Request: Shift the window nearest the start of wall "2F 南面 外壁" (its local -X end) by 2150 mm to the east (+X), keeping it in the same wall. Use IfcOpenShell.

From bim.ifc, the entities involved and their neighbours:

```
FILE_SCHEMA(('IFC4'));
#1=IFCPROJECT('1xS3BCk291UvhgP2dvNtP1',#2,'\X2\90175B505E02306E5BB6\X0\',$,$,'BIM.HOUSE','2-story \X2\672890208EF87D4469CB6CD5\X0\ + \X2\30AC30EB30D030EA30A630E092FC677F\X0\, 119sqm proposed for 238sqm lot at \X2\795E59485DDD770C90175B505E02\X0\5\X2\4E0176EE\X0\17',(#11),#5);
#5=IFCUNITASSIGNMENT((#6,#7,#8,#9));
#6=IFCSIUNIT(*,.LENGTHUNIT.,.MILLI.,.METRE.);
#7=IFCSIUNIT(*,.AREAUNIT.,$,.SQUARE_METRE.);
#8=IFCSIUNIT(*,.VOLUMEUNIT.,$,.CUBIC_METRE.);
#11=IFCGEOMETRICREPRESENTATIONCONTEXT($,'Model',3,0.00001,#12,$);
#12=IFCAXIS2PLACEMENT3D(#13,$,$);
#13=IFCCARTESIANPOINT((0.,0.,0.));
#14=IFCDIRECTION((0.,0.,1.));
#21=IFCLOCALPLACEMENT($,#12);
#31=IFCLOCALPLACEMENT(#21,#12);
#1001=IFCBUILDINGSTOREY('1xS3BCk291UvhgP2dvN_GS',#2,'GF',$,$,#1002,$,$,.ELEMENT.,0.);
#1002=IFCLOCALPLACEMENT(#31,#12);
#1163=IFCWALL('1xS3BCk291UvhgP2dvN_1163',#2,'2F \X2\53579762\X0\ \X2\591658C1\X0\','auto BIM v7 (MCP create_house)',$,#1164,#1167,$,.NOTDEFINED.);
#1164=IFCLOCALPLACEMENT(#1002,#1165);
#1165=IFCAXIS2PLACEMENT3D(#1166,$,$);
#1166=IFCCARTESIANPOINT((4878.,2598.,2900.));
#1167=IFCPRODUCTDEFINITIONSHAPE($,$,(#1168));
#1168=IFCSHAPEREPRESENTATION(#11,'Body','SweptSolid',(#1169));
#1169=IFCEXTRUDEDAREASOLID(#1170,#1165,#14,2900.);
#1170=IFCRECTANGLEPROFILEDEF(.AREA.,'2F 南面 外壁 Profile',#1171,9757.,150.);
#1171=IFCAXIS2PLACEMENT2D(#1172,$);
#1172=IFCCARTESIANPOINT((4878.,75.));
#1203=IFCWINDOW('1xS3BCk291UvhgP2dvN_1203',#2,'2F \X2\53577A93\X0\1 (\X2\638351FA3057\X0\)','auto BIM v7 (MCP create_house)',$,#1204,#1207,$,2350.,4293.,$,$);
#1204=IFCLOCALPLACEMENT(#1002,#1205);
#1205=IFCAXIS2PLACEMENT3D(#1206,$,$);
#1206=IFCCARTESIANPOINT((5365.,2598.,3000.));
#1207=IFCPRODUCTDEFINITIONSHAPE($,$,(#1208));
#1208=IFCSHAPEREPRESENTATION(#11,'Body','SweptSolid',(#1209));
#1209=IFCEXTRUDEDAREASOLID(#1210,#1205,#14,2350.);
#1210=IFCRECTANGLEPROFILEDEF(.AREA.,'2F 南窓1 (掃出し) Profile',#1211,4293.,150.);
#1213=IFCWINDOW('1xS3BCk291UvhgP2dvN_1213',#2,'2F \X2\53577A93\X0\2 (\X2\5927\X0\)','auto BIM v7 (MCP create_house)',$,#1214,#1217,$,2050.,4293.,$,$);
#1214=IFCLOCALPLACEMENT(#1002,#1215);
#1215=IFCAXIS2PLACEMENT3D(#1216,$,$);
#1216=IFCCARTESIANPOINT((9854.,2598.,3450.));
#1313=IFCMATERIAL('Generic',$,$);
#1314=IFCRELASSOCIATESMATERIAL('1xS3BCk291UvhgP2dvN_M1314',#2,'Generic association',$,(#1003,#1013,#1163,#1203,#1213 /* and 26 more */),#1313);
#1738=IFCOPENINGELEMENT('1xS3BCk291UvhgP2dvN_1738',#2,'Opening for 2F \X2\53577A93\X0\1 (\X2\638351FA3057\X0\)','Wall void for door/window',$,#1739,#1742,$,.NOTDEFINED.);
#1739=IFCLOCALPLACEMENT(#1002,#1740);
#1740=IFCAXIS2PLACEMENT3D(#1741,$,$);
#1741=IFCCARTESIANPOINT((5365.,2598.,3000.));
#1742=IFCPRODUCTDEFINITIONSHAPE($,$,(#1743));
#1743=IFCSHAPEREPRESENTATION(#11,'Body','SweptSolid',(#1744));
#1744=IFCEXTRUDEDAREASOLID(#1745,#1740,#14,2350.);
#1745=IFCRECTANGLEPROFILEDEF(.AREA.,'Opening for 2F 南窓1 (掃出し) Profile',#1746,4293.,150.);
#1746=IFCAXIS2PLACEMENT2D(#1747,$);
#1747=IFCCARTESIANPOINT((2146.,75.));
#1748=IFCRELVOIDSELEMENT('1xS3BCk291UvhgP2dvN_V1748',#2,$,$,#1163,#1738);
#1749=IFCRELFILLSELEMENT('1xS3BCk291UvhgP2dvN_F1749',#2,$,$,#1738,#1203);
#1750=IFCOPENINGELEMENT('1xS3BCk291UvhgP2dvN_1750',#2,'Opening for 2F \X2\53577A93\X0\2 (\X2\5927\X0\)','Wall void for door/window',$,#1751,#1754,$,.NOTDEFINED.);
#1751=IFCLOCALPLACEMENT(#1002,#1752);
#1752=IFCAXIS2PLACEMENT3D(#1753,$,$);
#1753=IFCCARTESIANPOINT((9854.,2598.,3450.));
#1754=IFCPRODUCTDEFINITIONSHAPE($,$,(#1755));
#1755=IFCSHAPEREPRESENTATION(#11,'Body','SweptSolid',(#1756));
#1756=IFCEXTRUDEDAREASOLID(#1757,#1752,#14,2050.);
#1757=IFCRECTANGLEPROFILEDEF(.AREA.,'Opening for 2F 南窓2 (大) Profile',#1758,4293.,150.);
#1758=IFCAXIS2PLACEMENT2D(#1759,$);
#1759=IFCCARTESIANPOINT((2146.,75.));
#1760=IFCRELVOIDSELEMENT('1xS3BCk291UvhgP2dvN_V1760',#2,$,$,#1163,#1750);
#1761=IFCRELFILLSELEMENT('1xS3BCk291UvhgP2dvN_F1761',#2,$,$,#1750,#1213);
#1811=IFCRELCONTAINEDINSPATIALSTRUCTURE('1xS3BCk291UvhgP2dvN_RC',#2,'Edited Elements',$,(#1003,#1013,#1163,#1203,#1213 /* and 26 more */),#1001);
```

```python
import ifcopenshell
import ifcopenshell.api.geometry
import ifcopenshell.util.placement
import ifcopenshell.util.unit

model = ifcopenshell.open("bim.ifc")
unit_scale = ifcopenshell.util.unit.calculate_unit_scale(model)

window = model.by_guid("1xS3BCk291UvhgP2dvN_1203")
opening = window.FillsVoids[0].RelatingOpeningElement
wall = opening.VoidsElements[0].RelatingBuildingElement

wall_matrix = ifcopenshell.util.placement.get_local_placement(wall.ObjectPlacement)
shift = wall_matrix[:3, 0] * 2.15 / unit_scale
before = ifcopenshell.util.placement.get_local_placement(window.ObjectPlacement)[:3, 3].copy()

# The window is not placed relative to its opening, so move both.
for product in (opening, window):
    matrix = ifcopenshell.util.placement.get_local_placement(product.ObjectPlacement)
    matrix[:3, 3] += shift
    ifcopenshell.api.geometry.edit_object_placement(model, product=product, matrix=matrix, is_si=False)

after = ifcopenshell.util.placement.get_local_placement(window.ObjectPlacement)[:3, 3]
print("window moved by", (after - before).round(3) + 0.0)

model.write("bim_updated.ifc")
```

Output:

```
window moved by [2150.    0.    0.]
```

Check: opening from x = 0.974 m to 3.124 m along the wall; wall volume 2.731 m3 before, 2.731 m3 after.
